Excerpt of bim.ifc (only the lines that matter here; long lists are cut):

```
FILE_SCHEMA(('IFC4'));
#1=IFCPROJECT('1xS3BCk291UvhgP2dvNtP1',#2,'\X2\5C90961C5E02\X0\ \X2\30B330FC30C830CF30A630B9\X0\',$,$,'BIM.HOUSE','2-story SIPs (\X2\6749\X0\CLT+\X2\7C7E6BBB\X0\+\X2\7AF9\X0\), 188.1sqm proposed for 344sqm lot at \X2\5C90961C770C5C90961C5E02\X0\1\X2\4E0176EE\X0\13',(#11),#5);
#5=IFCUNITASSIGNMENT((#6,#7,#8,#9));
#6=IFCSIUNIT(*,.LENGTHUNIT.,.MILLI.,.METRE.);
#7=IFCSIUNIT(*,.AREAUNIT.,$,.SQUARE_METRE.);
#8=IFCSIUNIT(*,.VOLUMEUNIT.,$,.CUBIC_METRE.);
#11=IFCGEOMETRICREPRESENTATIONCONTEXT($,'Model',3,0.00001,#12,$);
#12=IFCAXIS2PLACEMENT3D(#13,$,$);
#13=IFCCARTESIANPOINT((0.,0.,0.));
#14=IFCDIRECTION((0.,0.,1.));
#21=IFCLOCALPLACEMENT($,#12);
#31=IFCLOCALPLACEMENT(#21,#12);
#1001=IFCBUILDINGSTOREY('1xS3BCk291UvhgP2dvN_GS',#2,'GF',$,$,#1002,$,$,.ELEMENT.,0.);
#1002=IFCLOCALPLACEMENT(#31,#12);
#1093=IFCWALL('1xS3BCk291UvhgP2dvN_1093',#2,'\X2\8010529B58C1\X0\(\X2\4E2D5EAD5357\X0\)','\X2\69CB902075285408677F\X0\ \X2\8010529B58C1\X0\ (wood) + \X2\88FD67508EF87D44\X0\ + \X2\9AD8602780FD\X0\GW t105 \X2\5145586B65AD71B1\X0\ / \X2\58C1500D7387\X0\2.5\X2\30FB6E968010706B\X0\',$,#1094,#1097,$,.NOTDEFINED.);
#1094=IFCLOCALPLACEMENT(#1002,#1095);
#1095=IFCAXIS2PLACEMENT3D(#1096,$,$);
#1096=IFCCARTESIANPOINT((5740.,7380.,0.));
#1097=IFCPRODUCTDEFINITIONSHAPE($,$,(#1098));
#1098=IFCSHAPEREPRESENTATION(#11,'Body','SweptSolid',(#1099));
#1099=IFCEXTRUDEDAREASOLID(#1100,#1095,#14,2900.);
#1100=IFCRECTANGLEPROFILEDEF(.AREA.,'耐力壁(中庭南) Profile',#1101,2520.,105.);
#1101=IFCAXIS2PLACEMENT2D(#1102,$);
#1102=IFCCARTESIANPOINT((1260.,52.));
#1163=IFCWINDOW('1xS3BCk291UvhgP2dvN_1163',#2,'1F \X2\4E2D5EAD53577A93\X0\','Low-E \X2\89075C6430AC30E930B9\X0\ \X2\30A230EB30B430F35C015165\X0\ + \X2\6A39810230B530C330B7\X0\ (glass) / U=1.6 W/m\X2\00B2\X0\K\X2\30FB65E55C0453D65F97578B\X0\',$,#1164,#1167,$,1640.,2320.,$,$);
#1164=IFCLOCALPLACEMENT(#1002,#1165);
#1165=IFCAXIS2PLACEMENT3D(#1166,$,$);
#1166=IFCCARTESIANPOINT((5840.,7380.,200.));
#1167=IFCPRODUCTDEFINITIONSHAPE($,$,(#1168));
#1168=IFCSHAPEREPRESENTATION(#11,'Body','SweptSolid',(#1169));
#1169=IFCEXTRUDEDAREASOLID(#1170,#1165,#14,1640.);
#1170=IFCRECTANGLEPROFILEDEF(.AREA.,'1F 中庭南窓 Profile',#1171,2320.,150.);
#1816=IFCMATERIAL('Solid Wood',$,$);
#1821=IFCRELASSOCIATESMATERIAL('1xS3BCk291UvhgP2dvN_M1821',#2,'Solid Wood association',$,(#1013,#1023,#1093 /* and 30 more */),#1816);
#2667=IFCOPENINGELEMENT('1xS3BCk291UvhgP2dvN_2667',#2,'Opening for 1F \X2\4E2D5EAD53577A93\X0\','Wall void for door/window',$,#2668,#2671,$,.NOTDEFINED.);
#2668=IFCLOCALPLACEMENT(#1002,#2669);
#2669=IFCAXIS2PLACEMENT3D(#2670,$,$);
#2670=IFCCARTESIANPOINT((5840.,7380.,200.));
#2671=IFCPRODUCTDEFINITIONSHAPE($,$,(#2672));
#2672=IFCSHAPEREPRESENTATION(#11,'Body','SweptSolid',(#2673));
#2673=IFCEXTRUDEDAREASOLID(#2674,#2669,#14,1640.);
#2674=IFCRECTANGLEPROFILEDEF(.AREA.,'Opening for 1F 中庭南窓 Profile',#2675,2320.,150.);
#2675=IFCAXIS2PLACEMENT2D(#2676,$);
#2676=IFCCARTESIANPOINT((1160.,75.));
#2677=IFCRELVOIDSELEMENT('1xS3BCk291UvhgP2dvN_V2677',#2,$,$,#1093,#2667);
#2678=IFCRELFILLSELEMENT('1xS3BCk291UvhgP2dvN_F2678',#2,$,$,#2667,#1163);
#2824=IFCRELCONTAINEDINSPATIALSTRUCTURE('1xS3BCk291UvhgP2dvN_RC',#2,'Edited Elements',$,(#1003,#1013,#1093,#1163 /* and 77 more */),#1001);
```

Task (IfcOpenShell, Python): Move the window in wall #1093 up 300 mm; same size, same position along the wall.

```python
import numpy as np
import ifcopenshell
import ifcopenshell.api.geometry
import ifcopenshell.util.placement
import ifcopenshell.util.unit

model = ifcopenshell.open("bim.ifc")
unit_scale = ifcopenshell.util.unit.calculate_unit_scale(model)

window = model.by_id(1163)
opening = window.FillsVoids[0].RelatingOpeningElement
dz = 0.3 / unit_scale

shift = np.array([0.0, 0.0, dz])
# The window is not placed relative to its opening, so move both.
for product in (opening, window):
    matrix = ifcopenshell.util.placement.get_local_placement(product.ObjectPlacement)
    matrix[:3, 3] += shift
    ifcopenshell.api.geometry.edit_object_placement(model, product=product, matrix=matrix, is_si=False)

print(f"moved by {dz * unit_scale:+.3f} m")

model.write("bim_updated.ifc")
```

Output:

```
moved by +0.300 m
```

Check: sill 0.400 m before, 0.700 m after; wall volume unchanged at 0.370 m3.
